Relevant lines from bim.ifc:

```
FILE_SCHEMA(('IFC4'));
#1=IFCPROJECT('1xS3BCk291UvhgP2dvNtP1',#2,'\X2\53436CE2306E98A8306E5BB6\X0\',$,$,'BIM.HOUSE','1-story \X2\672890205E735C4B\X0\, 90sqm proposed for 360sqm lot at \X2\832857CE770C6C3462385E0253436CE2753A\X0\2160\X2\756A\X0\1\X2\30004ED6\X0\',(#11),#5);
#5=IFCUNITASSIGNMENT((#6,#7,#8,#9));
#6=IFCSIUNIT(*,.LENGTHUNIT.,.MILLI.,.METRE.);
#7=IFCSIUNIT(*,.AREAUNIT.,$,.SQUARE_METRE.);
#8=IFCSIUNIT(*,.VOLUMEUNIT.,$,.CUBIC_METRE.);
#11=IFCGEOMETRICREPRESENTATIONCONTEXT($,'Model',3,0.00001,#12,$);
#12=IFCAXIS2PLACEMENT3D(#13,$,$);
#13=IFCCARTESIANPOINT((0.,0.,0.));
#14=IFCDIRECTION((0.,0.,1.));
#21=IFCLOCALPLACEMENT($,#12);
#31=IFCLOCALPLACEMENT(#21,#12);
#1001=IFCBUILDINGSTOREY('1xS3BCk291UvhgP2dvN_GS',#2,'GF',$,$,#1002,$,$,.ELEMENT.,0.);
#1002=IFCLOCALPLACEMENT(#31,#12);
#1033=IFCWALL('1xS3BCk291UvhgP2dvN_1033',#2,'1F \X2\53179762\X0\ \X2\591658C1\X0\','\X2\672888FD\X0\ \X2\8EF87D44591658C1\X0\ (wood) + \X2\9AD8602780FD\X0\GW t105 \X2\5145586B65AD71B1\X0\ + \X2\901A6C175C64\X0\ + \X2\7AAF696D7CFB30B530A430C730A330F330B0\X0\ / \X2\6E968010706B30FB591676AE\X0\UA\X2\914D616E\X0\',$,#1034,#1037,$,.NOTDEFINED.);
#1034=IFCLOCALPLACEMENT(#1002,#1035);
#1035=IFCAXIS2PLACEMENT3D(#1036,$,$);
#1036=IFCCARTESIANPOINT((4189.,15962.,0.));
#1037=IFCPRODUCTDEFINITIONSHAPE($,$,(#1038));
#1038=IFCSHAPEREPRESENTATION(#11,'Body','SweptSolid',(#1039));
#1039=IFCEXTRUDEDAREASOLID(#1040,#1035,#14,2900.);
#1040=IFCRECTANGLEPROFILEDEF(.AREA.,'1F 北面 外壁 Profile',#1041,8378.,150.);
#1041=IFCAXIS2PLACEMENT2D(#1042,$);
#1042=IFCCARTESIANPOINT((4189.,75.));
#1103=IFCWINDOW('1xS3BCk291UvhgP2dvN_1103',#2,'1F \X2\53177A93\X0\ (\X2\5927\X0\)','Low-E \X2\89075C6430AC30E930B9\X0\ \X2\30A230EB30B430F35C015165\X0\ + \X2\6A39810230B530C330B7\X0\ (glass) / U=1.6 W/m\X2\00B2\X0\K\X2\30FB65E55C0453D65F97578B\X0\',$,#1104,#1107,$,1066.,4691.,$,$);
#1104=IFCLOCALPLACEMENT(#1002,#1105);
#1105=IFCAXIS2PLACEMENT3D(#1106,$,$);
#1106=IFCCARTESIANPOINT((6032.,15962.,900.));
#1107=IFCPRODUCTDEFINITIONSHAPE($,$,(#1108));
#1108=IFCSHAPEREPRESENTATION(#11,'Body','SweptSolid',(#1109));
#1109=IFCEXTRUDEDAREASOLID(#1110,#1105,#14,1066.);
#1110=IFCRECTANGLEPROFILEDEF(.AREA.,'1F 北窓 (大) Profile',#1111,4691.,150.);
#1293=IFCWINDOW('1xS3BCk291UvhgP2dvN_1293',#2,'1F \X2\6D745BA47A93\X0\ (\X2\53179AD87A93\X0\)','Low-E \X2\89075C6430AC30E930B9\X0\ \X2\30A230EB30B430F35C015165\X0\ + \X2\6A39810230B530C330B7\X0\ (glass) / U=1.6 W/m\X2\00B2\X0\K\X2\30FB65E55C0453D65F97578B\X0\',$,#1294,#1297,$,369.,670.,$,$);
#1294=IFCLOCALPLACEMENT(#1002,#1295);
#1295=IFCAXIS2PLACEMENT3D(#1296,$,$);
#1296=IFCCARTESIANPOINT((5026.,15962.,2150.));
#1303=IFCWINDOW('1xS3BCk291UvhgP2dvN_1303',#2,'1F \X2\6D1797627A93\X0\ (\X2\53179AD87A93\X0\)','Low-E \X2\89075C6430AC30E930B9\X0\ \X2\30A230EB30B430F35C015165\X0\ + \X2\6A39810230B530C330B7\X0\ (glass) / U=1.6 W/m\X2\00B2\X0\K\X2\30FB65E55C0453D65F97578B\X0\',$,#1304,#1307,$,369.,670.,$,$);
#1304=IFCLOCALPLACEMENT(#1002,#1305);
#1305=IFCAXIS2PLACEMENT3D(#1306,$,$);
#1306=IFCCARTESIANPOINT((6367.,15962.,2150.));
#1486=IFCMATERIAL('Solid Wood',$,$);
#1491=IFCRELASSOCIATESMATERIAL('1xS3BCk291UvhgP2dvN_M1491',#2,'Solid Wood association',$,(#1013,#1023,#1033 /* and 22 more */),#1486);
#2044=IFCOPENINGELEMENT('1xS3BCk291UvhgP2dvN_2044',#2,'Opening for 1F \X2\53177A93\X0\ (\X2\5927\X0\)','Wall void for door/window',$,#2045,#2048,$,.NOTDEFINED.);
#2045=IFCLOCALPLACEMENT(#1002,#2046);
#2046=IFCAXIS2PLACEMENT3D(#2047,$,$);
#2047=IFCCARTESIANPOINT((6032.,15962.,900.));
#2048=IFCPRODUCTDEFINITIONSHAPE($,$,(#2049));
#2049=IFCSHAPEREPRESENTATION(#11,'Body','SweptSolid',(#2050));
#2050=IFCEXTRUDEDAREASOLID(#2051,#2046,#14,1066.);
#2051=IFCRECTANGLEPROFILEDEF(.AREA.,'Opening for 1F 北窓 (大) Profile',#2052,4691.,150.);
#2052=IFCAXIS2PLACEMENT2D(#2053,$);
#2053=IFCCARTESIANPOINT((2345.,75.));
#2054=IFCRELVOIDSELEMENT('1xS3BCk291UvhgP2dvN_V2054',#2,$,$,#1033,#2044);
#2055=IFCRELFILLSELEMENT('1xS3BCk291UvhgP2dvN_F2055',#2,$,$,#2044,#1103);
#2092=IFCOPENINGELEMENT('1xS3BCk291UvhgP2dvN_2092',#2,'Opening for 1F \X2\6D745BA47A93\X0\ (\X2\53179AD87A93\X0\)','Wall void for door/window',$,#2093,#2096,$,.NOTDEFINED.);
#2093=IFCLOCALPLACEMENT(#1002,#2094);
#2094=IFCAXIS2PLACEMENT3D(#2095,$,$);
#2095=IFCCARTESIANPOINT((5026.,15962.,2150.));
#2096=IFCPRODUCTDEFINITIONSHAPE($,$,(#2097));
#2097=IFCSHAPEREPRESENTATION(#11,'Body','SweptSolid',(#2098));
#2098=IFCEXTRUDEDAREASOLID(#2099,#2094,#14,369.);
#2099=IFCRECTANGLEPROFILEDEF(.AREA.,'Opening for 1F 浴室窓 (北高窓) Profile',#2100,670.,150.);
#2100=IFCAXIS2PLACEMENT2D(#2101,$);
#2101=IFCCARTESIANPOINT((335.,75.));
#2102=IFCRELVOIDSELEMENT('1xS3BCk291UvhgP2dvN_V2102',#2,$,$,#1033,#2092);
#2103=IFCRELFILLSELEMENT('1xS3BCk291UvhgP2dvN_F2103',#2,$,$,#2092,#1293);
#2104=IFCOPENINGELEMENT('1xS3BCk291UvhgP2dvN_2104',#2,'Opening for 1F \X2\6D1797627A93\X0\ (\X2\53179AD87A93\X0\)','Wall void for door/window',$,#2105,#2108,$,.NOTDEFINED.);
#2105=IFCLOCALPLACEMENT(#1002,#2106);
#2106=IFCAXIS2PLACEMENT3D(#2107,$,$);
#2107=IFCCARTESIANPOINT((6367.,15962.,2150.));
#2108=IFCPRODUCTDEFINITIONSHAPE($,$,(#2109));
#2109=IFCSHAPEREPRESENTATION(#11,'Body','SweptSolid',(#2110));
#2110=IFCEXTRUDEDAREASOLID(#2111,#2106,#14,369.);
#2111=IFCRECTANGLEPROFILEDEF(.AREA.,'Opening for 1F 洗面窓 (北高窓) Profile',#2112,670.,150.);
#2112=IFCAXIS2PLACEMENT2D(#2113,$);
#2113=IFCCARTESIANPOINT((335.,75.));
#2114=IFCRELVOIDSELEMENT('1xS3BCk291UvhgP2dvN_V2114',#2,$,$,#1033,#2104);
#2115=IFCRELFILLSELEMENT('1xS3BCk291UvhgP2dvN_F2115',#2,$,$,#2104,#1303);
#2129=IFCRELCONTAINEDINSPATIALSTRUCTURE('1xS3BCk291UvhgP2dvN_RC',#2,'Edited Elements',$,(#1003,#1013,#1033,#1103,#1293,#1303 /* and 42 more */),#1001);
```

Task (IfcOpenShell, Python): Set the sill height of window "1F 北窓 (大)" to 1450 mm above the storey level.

```python
import numpy as np
import ifcopenshell
import ifcopenshell.api.geometry
import ifcopenshell.geom
import ifcopenshell.util.element
import ifcopenshell.util.placement
import ifcopenshell.util.shape
import ifcopenshell.util.unit

model = ifcopenshell.open("bim.ifc")
unit_scale = ifcopenshell.util.unit.calculate_unit_scale(model)

window = model.by_guid("1xS3BCk291UvhgP2dvN_1103")
opening = window.FillsVoids[0].RelatingOpeningElement
storey = ifcopenshell.util.element.get_container(window, ifc_class="IfcBuildingStorey")
level = ifcopenshell.util.placement.get_local_placement(storey.ObjectPlacement)[2, 3]

# The opening's origin need not be at the sill, so measure its lowest point.
shape = ifcopenshell.geom.create_shape(ifcopenshell.geom.settings(), opening)
bottom = ifcopenshell.util.shape.get_shape_bottom_elevation(shape, shape.geometry) / unit_scale
dz = level + 1.45 / unit_scale - bottom

shift = np.array([0.0, 0.0, dz])
# The window is not placed relative to its opening, so move both.
for product in (opening, window):
    matrix = ifcopenshell.util.placement.get_local_placement(product.ObjectPlacement)
    matrix[:3, 3] += shift
    ifcopenshell.api.geometry.edit_object_placement(model, product=product, matrix=matrix, is_si=False)

print(f"moved by {dz * unit_scale:+.3f} m")

model.write("bim_rev.ifc")
```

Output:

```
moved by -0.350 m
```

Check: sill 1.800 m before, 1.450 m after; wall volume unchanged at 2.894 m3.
